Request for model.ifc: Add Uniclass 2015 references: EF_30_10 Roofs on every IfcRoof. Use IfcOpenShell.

First a look at what the model holds.

```python
import ifcopenshell

model = ifcopenshell.open("model.ifc")
print(model.schema)
print("classifications:", [c.Name for c in model.by_type("IfcClassification")])
for ifc_class in ("IfcDoor", "IfcRoof", "IfcStair", "IfcWall", "IfcWindow"):
    print(ifc_class, len(model.by_type(ifc_class)))
```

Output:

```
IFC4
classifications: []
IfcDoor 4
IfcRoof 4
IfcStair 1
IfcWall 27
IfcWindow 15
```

```python
import ifcopenshell
import ifcopenshell.api.classification

model = ifcopenshell.open("model.ifc")

system = ifcopenshell.api.classification.add_classification(model, classification="Uniclass 2015")

codes = {
    "IfcRoof": ("EF_30_10", "Roofs"),
}
for ifc_class, (code, name) in codes.items():
    products = model.by_type(ifc_class)
    ifcopenshell.api.classification.add_reference(
        model, products=products, classification=system, identification=code, name=name
    )
    print(code, len(products))

model.write("model_v2.ifc")
```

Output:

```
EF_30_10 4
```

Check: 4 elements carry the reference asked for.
